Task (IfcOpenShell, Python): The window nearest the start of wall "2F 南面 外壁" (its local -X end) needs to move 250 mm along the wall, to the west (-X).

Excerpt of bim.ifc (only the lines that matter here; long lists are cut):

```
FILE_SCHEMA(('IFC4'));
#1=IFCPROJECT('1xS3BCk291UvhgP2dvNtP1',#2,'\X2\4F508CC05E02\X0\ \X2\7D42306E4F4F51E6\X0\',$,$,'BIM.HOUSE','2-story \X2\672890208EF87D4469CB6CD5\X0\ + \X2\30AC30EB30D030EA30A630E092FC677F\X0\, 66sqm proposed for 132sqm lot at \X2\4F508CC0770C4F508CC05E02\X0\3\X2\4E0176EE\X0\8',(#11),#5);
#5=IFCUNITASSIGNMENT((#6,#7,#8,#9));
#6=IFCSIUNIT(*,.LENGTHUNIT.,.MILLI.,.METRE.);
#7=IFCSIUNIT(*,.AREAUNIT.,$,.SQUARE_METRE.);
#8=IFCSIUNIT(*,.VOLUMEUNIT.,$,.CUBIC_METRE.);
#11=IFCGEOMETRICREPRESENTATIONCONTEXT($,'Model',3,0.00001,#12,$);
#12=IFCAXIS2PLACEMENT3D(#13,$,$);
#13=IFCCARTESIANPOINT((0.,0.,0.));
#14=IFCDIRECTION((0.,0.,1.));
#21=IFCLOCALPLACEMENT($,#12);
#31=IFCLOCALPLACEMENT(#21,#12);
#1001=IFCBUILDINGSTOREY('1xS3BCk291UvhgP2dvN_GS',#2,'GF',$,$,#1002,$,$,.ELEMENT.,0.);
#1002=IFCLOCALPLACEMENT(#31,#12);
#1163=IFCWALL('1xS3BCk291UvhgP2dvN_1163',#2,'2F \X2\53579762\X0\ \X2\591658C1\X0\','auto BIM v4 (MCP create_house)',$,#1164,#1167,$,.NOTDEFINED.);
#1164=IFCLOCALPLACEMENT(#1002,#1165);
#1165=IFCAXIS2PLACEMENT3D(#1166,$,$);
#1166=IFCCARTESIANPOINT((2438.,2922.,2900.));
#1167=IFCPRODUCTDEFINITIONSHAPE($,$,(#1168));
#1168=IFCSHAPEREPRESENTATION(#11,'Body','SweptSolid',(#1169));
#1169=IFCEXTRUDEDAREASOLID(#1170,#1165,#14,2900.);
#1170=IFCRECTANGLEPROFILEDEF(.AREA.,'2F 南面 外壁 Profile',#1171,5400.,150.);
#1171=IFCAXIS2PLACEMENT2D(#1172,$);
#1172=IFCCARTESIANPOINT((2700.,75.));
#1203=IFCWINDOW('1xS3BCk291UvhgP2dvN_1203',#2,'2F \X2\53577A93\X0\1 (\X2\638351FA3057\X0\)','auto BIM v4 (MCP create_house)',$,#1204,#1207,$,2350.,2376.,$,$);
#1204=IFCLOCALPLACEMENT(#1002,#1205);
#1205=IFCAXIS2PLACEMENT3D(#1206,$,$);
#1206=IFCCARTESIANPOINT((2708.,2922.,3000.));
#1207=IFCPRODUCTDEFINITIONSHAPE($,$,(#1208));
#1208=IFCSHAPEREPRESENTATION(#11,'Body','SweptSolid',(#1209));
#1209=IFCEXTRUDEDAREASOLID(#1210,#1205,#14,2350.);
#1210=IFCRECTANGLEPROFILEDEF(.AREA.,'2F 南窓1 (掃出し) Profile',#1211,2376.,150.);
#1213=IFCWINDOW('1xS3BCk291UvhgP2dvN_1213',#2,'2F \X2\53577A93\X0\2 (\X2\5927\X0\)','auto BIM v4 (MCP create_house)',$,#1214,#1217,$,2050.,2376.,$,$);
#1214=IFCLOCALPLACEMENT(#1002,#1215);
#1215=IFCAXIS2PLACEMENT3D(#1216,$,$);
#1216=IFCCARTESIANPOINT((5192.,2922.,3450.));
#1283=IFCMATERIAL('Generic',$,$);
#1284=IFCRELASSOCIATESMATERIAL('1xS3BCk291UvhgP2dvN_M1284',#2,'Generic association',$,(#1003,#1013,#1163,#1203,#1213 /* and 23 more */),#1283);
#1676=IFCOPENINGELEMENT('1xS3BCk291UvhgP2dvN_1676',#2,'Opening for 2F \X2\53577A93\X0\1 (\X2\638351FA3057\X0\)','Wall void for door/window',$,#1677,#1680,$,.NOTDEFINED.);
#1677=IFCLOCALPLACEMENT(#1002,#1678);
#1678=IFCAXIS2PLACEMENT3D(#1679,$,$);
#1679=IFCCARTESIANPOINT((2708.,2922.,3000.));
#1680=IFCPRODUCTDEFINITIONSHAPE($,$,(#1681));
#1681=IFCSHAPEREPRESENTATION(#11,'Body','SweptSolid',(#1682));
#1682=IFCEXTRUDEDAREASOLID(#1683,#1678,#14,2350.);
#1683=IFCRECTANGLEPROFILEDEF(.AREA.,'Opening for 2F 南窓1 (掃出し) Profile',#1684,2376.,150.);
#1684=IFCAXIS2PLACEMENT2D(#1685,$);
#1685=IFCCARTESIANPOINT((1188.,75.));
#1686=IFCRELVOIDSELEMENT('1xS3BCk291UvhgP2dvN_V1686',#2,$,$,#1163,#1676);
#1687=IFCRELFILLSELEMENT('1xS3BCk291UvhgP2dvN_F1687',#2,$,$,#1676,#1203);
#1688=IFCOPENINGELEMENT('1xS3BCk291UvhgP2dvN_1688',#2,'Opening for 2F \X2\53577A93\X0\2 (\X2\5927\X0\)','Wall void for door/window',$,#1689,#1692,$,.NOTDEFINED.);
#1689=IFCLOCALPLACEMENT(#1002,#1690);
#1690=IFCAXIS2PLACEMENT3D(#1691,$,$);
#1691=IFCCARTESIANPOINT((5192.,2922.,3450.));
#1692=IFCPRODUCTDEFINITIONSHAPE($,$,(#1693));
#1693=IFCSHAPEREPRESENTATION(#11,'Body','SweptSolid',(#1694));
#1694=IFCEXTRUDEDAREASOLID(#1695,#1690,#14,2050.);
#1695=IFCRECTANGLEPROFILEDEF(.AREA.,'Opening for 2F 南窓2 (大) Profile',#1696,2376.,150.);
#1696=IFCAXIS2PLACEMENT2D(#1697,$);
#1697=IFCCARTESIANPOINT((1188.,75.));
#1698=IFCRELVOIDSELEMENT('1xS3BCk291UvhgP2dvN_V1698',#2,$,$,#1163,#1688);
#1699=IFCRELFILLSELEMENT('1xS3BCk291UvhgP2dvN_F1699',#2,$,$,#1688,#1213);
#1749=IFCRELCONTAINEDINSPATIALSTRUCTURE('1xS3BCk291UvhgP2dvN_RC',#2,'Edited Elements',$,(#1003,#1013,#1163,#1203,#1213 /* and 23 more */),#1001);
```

```python
import ifcopenshell
import ifcopenshell.api.geometry
import ifcopenshell.util.placement
import ifcopenshell.util.unit

model = ifcopenshell.open("bim.ifc")
unit_scale = ifcopenshell.util.unit.calculate_unit_scale(model)

window = model.by_guid("1xS3BCk291UvhgP2dvN_1203")
opening = window.FillsVoids[0].RelatingOpeningElement
wall = opening.VoidsElements[0].RelatingBuildingElement

wall_matrix = ifcopenshell.util.placement.get_local_placement(wall.ObjectPlacement)
shift = wall_matrix[:3, 0] * -0.25 / unit_scale
before = ifcopenshell.util.placement.get_local_placement(window.ObjectPlacement)[:3, 3].copy()

# The window is not placed relative to its opening, so move both.
for product in (opening, window):
    matrix = ifcopenshell.util.placement.get_local_placement(product.ObjectPlacement)
    matrix[:3, 3] += shift
    ifcopenshell.api.geometry.edit_object_placement(model, product=product, matrix=matrix, is_si=False)

after = ifcopenshell.util.placement.get_local_placement(window.ObjectPlacement)[:3, 3]
print("window moved by", (after - before).round(3) + 0.0)

model.write("bim_edited.ifc")
```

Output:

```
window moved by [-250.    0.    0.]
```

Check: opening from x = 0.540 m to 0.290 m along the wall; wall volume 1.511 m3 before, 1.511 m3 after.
